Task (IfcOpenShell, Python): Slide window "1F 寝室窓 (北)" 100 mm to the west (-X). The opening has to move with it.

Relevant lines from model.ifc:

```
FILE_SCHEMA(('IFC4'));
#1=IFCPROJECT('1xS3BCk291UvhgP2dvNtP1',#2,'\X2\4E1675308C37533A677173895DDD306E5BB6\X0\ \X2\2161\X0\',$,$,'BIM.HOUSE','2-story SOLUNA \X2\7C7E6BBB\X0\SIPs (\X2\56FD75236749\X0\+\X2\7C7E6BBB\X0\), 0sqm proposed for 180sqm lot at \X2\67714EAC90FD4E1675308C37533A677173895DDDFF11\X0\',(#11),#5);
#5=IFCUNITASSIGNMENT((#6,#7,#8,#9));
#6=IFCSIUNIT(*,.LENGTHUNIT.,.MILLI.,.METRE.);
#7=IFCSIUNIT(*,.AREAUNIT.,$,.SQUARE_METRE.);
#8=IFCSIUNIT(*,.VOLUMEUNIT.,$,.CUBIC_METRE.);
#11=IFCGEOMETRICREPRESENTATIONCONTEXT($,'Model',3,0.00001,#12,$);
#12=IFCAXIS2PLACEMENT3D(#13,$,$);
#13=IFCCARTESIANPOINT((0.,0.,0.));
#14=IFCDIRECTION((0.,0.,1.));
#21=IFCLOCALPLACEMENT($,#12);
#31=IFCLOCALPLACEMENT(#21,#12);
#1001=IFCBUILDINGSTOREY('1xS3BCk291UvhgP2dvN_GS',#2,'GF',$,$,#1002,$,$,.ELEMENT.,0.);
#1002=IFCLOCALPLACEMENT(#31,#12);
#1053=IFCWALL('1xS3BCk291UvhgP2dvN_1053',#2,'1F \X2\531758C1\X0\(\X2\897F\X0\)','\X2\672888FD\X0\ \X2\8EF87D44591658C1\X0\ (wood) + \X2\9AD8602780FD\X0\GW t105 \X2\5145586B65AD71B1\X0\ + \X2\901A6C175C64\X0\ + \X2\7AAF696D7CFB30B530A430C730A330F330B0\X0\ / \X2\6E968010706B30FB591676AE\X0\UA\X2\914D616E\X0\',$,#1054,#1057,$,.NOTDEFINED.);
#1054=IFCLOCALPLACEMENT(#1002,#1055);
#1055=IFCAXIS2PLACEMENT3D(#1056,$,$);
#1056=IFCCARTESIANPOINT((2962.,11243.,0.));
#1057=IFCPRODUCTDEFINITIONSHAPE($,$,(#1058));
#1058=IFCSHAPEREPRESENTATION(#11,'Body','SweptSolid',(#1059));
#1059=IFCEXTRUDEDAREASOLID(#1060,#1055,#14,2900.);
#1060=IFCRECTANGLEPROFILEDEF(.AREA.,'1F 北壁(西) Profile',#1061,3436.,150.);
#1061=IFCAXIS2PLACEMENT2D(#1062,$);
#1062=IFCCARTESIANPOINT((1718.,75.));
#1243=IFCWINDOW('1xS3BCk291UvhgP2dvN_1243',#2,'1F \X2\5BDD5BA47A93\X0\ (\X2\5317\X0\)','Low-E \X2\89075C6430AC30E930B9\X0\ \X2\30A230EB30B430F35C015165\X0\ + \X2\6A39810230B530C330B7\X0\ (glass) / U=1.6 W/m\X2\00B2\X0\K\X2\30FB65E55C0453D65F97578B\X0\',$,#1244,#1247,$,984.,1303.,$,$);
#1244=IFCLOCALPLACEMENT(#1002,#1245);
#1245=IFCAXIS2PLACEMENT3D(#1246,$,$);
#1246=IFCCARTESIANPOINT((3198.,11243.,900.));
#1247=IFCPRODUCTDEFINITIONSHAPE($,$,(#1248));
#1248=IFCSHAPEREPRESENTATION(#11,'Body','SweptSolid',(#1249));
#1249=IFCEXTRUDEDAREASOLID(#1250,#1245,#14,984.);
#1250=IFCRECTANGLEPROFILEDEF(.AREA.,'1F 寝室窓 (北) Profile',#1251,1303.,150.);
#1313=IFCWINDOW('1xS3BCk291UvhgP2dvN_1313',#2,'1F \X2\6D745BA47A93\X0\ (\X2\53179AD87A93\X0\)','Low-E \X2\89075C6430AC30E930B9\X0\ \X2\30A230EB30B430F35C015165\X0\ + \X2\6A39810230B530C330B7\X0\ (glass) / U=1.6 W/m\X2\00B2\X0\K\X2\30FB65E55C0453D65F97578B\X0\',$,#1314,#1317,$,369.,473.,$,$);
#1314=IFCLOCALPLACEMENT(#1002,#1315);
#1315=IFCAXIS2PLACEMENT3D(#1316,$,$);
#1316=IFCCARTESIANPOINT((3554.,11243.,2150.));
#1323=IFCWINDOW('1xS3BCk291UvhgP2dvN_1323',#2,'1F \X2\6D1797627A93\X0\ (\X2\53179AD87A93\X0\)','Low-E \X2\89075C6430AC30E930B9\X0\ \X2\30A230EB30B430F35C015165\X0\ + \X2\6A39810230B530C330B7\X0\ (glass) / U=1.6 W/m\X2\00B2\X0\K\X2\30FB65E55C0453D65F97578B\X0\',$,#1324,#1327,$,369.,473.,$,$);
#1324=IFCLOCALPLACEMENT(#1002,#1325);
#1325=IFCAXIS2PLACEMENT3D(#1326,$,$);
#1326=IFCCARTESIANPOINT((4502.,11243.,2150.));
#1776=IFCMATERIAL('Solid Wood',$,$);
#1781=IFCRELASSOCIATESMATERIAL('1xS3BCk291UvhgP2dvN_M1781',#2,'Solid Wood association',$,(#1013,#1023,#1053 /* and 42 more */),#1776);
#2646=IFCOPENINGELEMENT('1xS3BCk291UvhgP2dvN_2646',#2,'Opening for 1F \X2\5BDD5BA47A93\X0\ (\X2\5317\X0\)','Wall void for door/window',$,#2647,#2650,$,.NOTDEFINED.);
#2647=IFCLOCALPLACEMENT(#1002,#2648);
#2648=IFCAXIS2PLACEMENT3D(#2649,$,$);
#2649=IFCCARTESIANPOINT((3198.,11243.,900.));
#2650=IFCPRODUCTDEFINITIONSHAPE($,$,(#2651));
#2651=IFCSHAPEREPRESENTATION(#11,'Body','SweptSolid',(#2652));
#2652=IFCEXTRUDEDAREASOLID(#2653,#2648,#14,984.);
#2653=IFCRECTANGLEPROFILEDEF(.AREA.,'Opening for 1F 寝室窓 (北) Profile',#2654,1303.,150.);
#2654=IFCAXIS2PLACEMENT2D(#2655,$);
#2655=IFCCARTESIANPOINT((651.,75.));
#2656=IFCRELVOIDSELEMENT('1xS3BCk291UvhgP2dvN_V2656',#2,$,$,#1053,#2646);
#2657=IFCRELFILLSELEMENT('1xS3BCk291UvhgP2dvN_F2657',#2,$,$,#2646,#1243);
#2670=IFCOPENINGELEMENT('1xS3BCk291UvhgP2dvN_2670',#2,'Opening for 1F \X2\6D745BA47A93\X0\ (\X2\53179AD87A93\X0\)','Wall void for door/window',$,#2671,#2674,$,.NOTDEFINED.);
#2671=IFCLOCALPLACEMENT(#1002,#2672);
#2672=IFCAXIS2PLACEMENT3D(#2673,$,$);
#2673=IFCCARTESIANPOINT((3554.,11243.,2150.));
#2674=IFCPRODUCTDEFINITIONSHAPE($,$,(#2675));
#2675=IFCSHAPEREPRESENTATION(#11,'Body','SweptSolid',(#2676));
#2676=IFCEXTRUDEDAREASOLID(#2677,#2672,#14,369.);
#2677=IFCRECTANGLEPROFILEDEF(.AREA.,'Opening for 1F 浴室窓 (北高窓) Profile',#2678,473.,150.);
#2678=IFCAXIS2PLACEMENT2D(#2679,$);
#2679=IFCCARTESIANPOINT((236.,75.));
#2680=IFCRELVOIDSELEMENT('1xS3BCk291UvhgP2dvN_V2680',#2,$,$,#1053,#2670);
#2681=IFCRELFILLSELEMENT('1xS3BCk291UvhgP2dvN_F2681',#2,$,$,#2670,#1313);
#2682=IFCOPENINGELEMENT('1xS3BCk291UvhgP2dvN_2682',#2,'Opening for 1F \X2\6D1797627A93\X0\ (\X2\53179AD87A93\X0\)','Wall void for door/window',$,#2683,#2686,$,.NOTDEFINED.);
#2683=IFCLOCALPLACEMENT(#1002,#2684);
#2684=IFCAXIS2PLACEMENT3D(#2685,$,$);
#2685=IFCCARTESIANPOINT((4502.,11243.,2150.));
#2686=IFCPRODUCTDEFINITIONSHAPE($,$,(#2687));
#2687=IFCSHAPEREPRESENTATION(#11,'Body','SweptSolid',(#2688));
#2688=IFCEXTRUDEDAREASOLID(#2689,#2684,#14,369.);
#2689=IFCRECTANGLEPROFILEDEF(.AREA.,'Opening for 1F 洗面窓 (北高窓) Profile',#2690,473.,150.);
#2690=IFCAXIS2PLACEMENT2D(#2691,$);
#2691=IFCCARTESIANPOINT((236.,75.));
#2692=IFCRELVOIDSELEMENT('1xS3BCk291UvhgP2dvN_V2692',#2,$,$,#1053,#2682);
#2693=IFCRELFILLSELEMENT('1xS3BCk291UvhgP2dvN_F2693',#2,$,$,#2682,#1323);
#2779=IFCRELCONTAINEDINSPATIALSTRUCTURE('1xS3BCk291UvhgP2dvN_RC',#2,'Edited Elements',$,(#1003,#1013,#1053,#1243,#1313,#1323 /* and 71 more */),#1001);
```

```python
import ifcopenshell
import ifcopenshell.api.geometry
import ifcopenshell.util.placement
import ifcopenshell.util.unit

model = ifcopenshell.open("model.ifc")
unit_scale = ifcopenshell.util.unit.calculate_unit_scale(model)

window = model.by_guid("1xS3BCk291UvhgP2dvN_1243")
opening = window.FillsVoids[0].RelatingOpeningElement
wall = opening.VoidsElements[0].RelatingBuildingElement

wall_matrix = ifcopenshell.util.placement.get_local_placement(wall.ObjectPlacement)
shift = wall_matrix[:3, 0] * -0.1 / unit_scale
before = ifcopenshell.util.placement.get_local_placement(window.ObjectPlacement)[:3, 3].copy()

# The window is not placed relative to its opening, so move both.
for product in (opening, window):
    matrix = ifcopenshell.util.placement.get_local_placement(product.ObjectPlacement)
    matrix[:3, 3] += shift
    ifcopenshell.api.geometry.edit_object_placement(model, product=product, matrix=matrix, is_si=False)

after = ifcopenshell.util.placement.get_local_placement(window.ObjectPlacement)[:3, 3]
print("window moved by", (after - before).round(3) + 0.0)

model.write("model_rev.ifc")
```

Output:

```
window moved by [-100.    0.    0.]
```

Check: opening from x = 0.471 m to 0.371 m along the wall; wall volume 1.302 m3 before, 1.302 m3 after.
